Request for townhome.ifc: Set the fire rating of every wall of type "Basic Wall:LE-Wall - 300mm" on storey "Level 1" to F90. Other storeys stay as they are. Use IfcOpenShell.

First a look at what the model holds.

```python
import ifcopenshell
import ifcopenshell.util.element

model = ifcopenshell.open("townhome.ifc")
print(model.schema)
storey = next(s for s in model.by_type("IfcBuildingStorey") if s.Name == "Level 1")
walls = [e for e in ifcopenshell.util.element.get_decomposition(storey) if e.is_a("IfcWall")]
seen = {}
for e in walls:
    element_type = ifcopenshell.util.element.get_type(e)
    key = (element_type.Name if element_type != e and element_type else None, ifcopenshell.util.element.get_pset(e, "Pset_WallCommon", "FireRating"))
    seen[key] = seen.get(key, 0) + 1
for (name, value), count in sorted(seen.items(), key=str):
    print(count, "x", name, "|", value)
```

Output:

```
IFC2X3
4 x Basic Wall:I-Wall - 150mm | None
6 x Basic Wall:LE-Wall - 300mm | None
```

```python
import ifcopenshell
import ifcopenshell.api.pset
import ifcopenshell.util.element

model = ifcopenshell.open("townhome.ifc")

storey = next(s for s in model.by_type("IfcBuildingStorey") if s.Name == "Level 1")
walls = [e for e in ifcopenshell.util.element.get_decomposition(storey) if e.is_a("IfcWall")]

count = 0
for e in walls:
    element_type = ifcopenshell.util.element.get_type(e)
    if element_type in (None, e) or element_type.Name != "Basic Wall:LE-Wall - 300mm":
        continue
    # add_pset returns the element's existing set when there is one.
    pset = ifcopenshell.api.pset.add_pset(model, product=e, name="Pset_WallCommon")
    ifcopenshell.api.pset.edit_pset(model, pset=pset, properties={"FireRating": "F90"})
    count += 1

print(count, "walls updated")

model.write("townhome-out.ifc")
```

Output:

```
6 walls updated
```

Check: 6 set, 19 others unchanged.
